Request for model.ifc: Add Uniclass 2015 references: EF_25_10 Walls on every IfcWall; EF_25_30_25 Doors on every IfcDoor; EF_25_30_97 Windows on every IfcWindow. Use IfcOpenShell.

First a look at what the model holds.

```python
import ifcopenshell

model = ifcopenshell.open("model.ifc")
print(model.schema)
print("classifications:", [c.Name for c in model.by_type("IfcClassification")])
for ifc_class in ("IfcDoor", "IfcRoof", "IfcStair", "IfcWall", "IfcWindow"):
    print(ifc_class, len(model.by_type(ifc_class)))
```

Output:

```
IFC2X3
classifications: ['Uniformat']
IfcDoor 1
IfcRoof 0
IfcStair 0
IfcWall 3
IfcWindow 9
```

```python
import ifcopenshell
import ifcopenshell.api.classification

model = ifcopenshell.open("model.ifc")

# IFC2X3 requires Source and Edition and has no link from the project to the system.
system = model.create_entity("IfcClassification", Source="NBS", Edition="2015", Name="Uniclass 2015")

codes = {
    "IfcWall": ("EF_25_10", "Walls"),
    "IfcDoor": ("EF_25_30_25", "Doors"),
    "IfcWindow": ("EF_25_30_97", "Windows"),
}
for ifc_class, (code, name) in codes.items():
    products = model.by_type(ifc_class)
    ifcopenshell.api.classification.add_reference(
        model, products=products, classification=system, identification=code, name=name
    )
    print(code, len(products))

model.write("model_v2.ifc")
```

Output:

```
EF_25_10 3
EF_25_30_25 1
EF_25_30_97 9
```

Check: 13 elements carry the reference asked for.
